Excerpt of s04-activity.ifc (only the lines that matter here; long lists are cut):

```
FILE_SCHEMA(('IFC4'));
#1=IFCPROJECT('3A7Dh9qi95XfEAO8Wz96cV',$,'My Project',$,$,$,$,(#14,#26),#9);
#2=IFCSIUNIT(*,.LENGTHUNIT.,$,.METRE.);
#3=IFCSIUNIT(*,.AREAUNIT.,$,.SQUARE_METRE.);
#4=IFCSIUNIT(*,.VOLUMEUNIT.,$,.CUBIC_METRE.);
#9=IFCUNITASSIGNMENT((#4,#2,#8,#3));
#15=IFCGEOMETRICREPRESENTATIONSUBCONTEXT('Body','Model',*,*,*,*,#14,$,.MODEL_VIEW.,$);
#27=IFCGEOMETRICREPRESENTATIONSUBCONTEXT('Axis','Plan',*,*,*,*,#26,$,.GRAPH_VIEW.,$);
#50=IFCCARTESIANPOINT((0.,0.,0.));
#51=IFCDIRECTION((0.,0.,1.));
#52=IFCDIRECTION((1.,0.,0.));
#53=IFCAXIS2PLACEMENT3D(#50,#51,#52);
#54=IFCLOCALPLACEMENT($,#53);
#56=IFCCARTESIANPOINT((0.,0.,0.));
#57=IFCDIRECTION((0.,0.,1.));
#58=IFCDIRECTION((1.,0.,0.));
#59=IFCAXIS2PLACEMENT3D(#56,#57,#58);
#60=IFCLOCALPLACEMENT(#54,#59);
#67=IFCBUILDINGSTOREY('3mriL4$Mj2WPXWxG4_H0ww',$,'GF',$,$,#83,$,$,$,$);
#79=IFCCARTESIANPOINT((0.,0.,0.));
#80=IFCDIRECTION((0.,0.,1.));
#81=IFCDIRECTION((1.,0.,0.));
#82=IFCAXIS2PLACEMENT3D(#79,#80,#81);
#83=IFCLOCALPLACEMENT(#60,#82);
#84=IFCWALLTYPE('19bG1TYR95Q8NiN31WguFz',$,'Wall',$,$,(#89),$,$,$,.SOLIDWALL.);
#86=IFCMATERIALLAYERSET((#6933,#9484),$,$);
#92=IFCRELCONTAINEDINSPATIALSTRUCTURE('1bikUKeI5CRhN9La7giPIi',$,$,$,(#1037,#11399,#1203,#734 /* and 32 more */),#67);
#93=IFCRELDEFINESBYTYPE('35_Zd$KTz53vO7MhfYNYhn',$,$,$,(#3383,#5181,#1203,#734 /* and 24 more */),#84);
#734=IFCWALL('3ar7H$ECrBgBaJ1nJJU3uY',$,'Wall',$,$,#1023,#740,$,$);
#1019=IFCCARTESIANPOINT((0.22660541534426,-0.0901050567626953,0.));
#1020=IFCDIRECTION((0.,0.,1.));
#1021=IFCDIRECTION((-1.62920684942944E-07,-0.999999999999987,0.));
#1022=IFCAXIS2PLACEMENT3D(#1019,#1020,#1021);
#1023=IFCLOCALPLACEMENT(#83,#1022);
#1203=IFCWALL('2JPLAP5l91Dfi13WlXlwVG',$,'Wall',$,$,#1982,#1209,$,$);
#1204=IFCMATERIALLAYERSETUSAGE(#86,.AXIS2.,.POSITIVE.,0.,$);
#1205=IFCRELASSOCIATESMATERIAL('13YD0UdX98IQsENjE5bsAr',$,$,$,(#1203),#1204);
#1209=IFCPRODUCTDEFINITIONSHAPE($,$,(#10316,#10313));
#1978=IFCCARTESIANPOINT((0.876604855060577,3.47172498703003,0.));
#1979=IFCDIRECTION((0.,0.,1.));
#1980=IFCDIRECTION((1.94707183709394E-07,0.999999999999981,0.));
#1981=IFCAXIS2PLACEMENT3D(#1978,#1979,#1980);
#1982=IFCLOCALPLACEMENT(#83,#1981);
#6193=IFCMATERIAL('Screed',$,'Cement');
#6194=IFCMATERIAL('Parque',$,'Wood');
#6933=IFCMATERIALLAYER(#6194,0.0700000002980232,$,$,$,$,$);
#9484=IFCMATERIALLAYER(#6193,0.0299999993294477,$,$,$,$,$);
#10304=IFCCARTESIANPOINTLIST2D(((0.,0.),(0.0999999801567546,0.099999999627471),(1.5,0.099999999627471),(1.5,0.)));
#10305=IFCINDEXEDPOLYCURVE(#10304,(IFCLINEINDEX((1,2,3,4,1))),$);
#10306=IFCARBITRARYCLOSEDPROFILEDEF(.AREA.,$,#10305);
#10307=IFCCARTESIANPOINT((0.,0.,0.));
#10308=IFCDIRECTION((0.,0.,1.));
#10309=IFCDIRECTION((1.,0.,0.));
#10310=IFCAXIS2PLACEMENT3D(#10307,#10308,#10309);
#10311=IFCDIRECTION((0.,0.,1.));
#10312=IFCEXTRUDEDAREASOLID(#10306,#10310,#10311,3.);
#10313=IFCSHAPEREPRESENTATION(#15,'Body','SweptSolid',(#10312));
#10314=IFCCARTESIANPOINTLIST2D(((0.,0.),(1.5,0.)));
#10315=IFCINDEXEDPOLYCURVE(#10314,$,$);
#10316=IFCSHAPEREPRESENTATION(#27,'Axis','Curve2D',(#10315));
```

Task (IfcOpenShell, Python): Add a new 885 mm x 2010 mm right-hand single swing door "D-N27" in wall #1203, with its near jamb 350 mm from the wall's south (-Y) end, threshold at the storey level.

```python
import numpy as np
import ifcopenshell
import ifcopenshell.api.feature
import ifcopenshell.api.geometry
import ifcopenshell.api.root
import ifcopenshell.api.spatial
import ifcopenshell.geom
import ifcopenshell.util.element
import ifcopenshell.util.placement
import ifcopenshell.util.representation
import ifcopenshell.util.shape
import ifcopenshell.util.unit

model = ifcopenshell.open("s04-activity.ifc")
unit_scale = ifcopenshell.util.unit.calculate_unit_scale(model)
settings = ifcopenshell.geom.settings()


def volume(element):
    """Net volume in cubic metres, openings subtracted."""
    shape = ifcopenshell.geom.create_shape(settings, element)
    return ifcopenshell.util.shape.get_volume(shape.geometry)


wall = model.by_id(1203)
storey = ifcopenshell.util.element.get_container(wall, ifc_class="IfcBuildingStorey")
context = ifcopenshell.util.representation.get_context(model, "Model", "Body", "MODEL_VIEW")
before = volume(wall)

width, height, from_end, sill = 0.885, 2.01, 0.35, 0.0  # metres

# The wall runs along its own X axis, and the end named is its -X end.
wall_shape = ifcopenshell.geom.create_shape(settings, wall)
x, y, z = ifcopenshell.util.shape.get_vertices(wall_shape.geometry).T
start = x.min() + from_end
face, thickness = float(y.min()), float(y.max() - y.min())
wall_matrix = ifcopenshell.util.placement.get_local_placement(wall.ObjectPlacement)
level = ifcopenshell.util.placement.get_local_placement(storey.ObjectPlacement)[2, 3]


def in_wall(x, y):
    """Placement at x, y metres in the wall's axes, at sill height."""
    matrix = wall_matrix.copy()
    matrix[:, 3] = wall_matrix @ np.array([x / unit_scale, y / unit_scale, 0.0, 1.0])
    matrix[2, 3] = level + sill / unit_scale
    return matrix


# Opening: a box that overshoots both wall faces by 50 mm.
opening = ifcopenshell.api.root.create_entity(model, ifc_class="IfcOpeningElement", predefined_type="OPENING")
box = ifcopenshell.api.geometry.add_wall_representation(
    model, context=context, length=width, height=height, thickness=thickness + 0.1
)
ifcopenshell.api.geometry.assign_representation(model, product=opening, representation=box)
ifcopenshell.api.geometry.edit_object_placement(model, product=opening, matrix=in_wall(start, face - 0.05), is_si=False)
ifcopenshell.api.feature.add_feature(model, feature=opening, element=wall)

door = ifcopenshell.api.root.create_entity(model, ifc_class="IfcDoor", name="D-N27", predefined_type="DOOR")
door.OverallWidth, door.OverallHeight = width / unit_scale, height / unit_scale
door.OperationType = "SINGLE_SWING_RIGHT"
body = ifcopenshell.api.geometry.add_door_representation(
    model,
    context=context,
    overall_width=door.OverallWidth,
    overall_height=door.OverallHeight,
    operation_type="SINGLE_SWING_RIGHT",
    lining_properties={"LiningDepth": thickness / unit_scale, "ThresholdDepth": thickness / unit_scale},
)
ifcopenshell.api.geometry.assign_representation(model, product=door, representation=body)
ifcopenshell.api.spatial.assign_container(model, products=[door], relating_structure=storey)
ifcopenshell.api.feature.add_filling(model, opening=opening, element=door)

# The lining spans the wall, so the door starts at the wall face.
ifcopenshell.api.geometry.edit_object_placement(model, product=door, matrix=in_wall(start, face), is_si=False)

after = volume(wall)

print(f"wall volume {before:.3f} -> {after:.3f} m3")

model.write("s04-activity_updated.ifc")
```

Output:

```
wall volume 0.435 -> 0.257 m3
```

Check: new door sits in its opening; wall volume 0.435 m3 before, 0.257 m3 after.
